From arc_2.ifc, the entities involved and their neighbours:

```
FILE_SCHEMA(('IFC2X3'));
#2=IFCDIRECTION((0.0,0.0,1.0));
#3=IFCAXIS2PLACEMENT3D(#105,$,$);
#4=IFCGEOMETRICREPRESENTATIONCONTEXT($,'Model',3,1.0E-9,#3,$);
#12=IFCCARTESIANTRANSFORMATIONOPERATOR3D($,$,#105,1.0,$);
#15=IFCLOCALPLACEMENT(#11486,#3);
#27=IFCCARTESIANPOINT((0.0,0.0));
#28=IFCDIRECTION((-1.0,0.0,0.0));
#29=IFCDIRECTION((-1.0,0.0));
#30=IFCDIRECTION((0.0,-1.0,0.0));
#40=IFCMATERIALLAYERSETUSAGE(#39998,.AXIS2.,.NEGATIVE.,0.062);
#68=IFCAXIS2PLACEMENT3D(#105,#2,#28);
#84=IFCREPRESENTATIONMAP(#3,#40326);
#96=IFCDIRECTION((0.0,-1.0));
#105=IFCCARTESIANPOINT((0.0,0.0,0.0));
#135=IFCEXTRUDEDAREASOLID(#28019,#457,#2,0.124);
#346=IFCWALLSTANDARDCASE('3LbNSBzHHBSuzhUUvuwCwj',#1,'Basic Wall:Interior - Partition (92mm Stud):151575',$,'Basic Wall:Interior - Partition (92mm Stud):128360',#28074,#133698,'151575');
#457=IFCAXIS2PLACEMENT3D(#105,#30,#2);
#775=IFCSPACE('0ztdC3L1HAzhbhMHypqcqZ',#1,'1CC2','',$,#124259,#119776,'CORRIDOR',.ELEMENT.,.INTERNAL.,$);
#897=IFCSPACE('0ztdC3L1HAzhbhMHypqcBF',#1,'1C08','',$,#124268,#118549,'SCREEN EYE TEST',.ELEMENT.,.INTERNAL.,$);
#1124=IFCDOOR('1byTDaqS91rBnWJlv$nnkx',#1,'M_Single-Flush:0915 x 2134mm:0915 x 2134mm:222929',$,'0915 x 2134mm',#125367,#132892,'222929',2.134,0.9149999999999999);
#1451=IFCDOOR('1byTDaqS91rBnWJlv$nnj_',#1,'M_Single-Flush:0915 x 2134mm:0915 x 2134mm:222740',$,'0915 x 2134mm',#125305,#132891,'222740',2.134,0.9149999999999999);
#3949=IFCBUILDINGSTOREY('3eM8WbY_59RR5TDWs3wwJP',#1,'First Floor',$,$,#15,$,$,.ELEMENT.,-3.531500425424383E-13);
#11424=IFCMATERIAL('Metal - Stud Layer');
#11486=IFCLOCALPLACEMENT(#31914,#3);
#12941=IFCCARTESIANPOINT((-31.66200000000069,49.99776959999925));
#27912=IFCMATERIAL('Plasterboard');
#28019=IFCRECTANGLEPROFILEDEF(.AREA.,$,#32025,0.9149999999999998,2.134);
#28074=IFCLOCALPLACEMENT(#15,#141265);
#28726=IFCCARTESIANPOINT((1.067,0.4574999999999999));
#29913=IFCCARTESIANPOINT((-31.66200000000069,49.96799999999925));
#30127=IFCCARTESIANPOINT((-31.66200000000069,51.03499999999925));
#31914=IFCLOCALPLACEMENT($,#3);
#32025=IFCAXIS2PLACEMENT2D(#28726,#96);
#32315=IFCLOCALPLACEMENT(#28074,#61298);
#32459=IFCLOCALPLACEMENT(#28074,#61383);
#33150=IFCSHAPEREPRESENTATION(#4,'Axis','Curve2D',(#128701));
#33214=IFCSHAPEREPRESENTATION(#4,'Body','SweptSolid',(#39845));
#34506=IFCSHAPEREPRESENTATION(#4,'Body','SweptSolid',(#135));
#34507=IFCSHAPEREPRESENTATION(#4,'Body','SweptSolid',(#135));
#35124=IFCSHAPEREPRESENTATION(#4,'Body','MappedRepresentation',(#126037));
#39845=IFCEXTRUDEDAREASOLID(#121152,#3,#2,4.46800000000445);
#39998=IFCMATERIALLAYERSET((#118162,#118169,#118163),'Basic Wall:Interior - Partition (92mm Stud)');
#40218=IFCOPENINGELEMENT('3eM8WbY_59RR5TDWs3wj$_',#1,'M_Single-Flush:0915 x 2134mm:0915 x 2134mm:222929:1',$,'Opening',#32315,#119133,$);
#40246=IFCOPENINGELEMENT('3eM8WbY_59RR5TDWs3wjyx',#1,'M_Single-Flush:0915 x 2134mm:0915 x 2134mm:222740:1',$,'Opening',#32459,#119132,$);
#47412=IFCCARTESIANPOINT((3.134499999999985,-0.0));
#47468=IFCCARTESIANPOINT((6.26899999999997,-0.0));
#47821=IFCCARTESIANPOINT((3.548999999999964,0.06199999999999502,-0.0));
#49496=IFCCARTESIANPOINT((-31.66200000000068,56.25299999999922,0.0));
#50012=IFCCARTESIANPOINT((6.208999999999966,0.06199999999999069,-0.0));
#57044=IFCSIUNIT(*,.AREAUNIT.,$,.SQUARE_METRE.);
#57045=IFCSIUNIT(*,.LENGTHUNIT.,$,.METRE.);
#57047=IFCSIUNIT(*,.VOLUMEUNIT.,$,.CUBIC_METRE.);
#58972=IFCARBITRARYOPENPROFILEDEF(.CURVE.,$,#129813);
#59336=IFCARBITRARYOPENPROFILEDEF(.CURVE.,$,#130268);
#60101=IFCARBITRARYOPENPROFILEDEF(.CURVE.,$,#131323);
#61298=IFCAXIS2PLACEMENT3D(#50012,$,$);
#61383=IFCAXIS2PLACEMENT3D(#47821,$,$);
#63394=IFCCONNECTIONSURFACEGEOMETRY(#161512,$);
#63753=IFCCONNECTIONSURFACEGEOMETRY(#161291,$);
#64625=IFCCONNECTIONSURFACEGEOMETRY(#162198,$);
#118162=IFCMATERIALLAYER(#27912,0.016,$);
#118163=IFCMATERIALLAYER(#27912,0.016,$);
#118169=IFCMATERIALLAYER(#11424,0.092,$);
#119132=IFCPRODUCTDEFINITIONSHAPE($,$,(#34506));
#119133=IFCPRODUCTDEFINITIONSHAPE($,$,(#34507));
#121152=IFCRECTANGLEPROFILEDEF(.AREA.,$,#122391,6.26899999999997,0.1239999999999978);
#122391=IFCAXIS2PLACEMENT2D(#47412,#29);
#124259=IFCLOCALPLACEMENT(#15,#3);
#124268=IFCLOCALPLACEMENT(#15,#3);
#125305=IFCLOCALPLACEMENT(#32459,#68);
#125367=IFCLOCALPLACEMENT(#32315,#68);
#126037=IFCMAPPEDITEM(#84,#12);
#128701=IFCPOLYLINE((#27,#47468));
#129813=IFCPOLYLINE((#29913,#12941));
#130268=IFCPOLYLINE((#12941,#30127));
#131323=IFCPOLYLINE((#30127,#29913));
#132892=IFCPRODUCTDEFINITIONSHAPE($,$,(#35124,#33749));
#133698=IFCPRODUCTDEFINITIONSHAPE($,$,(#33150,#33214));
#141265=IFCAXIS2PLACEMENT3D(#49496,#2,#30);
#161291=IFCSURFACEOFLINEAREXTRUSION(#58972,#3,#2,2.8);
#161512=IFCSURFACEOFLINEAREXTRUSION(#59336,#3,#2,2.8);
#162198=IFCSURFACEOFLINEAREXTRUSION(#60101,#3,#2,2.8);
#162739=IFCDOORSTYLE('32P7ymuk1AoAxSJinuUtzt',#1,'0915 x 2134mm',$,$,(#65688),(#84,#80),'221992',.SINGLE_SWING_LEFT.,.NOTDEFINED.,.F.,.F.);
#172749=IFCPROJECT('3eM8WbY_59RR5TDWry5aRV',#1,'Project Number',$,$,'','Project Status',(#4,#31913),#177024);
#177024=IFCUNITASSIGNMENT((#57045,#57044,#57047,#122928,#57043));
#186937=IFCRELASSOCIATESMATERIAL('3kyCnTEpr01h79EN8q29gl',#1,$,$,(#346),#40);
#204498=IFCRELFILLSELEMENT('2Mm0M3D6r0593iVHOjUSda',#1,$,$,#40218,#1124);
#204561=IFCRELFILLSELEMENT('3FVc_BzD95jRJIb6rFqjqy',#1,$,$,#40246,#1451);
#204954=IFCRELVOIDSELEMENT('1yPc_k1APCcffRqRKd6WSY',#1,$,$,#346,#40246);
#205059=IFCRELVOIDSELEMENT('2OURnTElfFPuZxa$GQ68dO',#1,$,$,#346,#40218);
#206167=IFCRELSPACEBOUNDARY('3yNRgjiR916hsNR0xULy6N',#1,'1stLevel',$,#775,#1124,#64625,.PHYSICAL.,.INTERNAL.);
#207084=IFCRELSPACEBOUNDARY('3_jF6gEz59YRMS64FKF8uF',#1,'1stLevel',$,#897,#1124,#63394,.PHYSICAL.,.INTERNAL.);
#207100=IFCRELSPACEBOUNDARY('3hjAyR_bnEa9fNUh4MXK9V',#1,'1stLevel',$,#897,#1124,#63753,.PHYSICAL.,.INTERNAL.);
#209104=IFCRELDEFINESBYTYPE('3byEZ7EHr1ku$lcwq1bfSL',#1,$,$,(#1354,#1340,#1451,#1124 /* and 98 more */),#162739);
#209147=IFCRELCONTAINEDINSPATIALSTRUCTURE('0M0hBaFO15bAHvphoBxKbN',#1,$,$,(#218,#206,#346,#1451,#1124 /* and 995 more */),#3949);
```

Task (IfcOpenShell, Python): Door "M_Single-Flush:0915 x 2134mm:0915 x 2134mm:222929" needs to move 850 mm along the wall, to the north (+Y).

```python
import numpy as np
import ifcopenshell
import ifcopenshell.api.geometry
import ifcopenshell.util.placement

model = ifcopenshell.open("arc_2.ifc")

door = model.by_guid("1byTDaqS91rBnWJlv$nnkx")
opening = door.FillsVoids[0].RelatingOpeningElement
wall = opening.VoidsElements[0].RelatingBuildingElement

wall_matrix = ifcopenshell.util.placement.get_local_placement(wall.ObjectPlacement)
shift = wall_matrix[:3, 0] * -0.85
before = ifcopenshell.util.placement.get_local_placement(door.ObjectPlacement)[:3, 3].copy()

# The door is placed relative to its opening, so it follows when the opening moves.
matrix = ifcopenshell.util.placement.get_local_placement(opening.ObjectPlacement)
matrix[:3, 3] += shift
ifcopenshell.api.geometry.edit_object_placement(
    model, product=opening, matrix=matrix, is_si=False, should_transform_children=True
)

# Space boundary surfaces are stored in each space's coordinates; move them too.
for rel in door.ProvidesBoundaries:
    if not rel.ConnectionGeometry:
        continue
    surface = rel.ConnectionGeometry.SurfaceOnRelatingElement
    space_matrix = ifcopenshell.util.placement.get_local_placement(rel.RelatingSpace.ObjectPlacement)
    point = np.array(surface.Position.Location.Coordinates) + space_matrix[:3, :3].T @ shift
    surface.Position = model.createIfcAxis2Placement3D(
        model.createIfcCartesianPoint(point.tolist()), surface.Position.Axis, surface.Position.RefDirection
    )

after = ifcopenshell.util.placement.get_local_placement(door.ObjectPlacement)[:3, 3]
print("door moved by", (after - before).round(3) + 0.0)

model.write("arc_2_edited.ifc")
```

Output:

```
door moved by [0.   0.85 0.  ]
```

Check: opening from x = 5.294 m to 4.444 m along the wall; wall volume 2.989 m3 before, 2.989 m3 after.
